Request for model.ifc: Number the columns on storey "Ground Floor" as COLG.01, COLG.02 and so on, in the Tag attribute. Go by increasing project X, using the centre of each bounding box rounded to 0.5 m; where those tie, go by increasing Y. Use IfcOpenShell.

First a look at what the model holds.

```python
import ifcopenshell
import ifcopenshell.util.element
import ifcopenshell.util.placement

model = ifcopenshell.open("model.ifc")
print(model.schema)
storey = next(s for s in model.by_type("IfcBuildingStorey") if s.Name == "Ground Floor")
columns = [e for e in ifcopenshell.util.element.get_decomposition(storey) if e.is_a("IfcColumn")]
for e in sorted(columns, key=lambda e: e.id()):
    origin = ifcopenshell.util.placement.get_local_placement(e.ObjectPlacement)[:3, 3]
    print(e.id(), e.Tag, e.Name, origin.round(2) + 0.0, sep=" | ")
```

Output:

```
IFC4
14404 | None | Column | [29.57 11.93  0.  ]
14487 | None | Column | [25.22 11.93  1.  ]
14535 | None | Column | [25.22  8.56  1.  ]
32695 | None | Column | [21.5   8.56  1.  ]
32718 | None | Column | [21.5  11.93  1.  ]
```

```python
import ifcopenshell
import ifcopenshell.geom
import ifcopenshell.util.element
import ifcopenshell.util.shape

model = ifcopenshell.open("model.ifc")
settings = ifcopenshell.geom.settings()
settings.set("use-world-coords", True)


def centre(element):
    shape = ifcopenshell.geom.create_shape(settings, element)
    return ifcopenshell.util.shape.get_bbox_centroid(shape.geometry)


storey = next(s for s in model.by_type("IfcBuildingStorey") if s.Name == "Ground Floor")
columns = [e for e in ifcopenshell.util.element.get_decomposition(storey) if e.is_a("IfcColumn")]

# Insertion points can sit at a corner or the storey origin, so sort by the geometry (in metres).
centres = {e: centre(e) for e in columns}
columns.sort(key=lambda e: (round(centres[e][0] / 0.5), centres[e][1]))

for i, e in enumerate(columns, start=1):
    number = f"COLG.{i:02d}"
    e.Tag = number
    print(e.id(), number)

model.write("model_edited.ifc")
```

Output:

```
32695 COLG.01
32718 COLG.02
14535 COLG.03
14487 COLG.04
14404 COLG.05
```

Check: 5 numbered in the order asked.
